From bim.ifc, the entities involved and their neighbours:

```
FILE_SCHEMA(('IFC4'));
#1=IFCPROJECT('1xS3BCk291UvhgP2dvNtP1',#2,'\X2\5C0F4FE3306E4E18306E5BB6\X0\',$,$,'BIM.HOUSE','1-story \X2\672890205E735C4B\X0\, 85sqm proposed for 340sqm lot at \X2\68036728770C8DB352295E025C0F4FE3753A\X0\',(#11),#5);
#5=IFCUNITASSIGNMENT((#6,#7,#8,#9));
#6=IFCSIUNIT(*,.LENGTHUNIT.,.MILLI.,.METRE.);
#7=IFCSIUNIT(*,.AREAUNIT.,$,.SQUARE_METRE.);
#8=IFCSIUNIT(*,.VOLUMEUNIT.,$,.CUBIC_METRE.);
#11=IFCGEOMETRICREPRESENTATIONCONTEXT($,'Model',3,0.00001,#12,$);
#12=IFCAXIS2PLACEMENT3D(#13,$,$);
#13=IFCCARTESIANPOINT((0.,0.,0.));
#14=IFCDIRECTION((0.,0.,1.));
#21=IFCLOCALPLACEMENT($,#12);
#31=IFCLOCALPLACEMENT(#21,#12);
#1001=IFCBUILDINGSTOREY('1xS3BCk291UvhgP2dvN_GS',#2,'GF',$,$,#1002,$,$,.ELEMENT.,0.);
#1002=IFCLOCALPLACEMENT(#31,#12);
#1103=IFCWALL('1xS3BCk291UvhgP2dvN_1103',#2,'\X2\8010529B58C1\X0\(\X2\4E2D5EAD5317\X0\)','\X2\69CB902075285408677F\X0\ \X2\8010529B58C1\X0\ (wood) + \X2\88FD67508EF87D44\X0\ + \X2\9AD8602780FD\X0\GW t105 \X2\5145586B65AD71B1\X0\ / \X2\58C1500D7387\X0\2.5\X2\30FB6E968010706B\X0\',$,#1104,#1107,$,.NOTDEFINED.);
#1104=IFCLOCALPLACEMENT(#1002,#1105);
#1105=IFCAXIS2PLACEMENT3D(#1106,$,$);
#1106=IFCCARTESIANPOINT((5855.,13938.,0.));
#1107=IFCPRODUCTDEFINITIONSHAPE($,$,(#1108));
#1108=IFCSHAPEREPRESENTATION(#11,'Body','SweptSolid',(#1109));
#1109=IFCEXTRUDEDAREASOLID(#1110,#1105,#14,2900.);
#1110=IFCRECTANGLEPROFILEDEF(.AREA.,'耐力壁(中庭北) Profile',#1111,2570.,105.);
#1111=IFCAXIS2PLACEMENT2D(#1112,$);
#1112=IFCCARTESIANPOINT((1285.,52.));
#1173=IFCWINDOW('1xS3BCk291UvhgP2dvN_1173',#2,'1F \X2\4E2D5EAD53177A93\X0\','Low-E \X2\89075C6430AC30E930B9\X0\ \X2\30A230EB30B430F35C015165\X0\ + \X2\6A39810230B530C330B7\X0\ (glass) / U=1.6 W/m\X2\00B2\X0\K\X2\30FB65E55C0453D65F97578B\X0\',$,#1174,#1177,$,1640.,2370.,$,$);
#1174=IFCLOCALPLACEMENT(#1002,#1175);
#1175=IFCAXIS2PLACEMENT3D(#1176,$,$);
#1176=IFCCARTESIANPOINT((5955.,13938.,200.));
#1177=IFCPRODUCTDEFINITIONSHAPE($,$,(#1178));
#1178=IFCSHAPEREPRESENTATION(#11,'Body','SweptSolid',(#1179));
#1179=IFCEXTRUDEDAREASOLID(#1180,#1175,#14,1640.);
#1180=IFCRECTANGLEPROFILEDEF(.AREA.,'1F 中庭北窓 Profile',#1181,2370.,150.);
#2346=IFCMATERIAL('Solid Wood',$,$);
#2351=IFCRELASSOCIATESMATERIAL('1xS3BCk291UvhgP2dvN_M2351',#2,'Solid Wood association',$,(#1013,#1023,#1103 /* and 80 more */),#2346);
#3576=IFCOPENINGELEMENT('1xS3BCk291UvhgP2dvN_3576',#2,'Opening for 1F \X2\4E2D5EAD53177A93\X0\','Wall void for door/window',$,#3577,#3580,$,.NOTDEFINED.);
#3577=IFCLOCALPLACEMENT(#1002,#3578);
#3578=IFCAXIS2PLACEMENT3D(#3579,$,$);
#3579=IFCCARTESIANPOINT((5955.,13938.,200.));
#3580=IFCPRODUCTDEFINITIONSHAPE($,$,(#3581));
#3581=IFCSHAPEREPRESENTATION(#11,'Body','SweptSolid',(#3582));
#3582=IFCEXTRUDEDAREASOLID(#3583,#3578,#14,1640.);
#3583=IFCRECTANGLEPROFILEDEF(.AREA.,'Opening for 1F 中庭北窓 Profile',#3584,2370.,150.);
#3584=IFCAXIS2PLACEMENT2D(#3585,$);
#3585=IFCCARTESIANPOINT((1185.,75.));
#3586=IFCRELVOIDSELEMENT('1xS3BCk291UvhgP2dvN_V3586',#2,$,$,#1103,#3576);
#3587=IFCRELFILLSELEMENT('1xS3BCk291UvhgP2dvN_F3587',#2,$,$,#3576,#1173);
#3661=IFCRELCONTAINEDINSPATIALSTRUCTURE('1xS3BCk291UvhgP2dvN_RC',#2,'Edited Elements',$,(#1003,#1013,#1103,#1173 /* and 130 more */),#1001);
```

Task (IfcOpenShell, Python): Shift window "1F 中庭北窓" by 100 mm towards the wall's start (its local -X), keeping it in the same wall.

```python
import ifcopenshell
import ifcopenshell.api.geometry
import ifcopenshell.util.placement

model = ifcopenshell.open("bim.ifc")

window = model.by_guid("1xS3BCk291UvhgP2dvN_1173")
opening = window.FillsVoids[0].RelatingOpeningElement
wall = opening.VoidsElements[0].RelatingBuildingElement

wall_matrix = ifcopenshell.util.placement.get_local_placement(wall.ObjectPlacement)
shift = wall_matrix[:3, 0] * -100.0
before = ifcopenshell.util.placement.get_local_placement(window.ObjectPlacement)[:3, 3].copy()

# The window is not placed relative to its opening, so move both.
for product in (opening, window):
    matrix = ifcopenshell.util.placement.get_local_placement(product.ObjectPlacement)
    matrix[:3, 3] += shift
    ifcopenshell.api.geometry.edit_object_placement(model, product=product, matrix=matrix, is_si=False)

after = ifcopenshell.util.placement.get_local_placement(window.ObjectPlacement)[:3, 3]
print("window moved by", (after - before).round(3) + 0.0)

model.write("bim_updated.ifc")
```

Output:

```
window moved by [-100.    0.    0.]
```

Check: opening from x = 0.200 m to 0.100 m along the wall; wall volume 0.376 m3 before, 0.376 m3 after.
